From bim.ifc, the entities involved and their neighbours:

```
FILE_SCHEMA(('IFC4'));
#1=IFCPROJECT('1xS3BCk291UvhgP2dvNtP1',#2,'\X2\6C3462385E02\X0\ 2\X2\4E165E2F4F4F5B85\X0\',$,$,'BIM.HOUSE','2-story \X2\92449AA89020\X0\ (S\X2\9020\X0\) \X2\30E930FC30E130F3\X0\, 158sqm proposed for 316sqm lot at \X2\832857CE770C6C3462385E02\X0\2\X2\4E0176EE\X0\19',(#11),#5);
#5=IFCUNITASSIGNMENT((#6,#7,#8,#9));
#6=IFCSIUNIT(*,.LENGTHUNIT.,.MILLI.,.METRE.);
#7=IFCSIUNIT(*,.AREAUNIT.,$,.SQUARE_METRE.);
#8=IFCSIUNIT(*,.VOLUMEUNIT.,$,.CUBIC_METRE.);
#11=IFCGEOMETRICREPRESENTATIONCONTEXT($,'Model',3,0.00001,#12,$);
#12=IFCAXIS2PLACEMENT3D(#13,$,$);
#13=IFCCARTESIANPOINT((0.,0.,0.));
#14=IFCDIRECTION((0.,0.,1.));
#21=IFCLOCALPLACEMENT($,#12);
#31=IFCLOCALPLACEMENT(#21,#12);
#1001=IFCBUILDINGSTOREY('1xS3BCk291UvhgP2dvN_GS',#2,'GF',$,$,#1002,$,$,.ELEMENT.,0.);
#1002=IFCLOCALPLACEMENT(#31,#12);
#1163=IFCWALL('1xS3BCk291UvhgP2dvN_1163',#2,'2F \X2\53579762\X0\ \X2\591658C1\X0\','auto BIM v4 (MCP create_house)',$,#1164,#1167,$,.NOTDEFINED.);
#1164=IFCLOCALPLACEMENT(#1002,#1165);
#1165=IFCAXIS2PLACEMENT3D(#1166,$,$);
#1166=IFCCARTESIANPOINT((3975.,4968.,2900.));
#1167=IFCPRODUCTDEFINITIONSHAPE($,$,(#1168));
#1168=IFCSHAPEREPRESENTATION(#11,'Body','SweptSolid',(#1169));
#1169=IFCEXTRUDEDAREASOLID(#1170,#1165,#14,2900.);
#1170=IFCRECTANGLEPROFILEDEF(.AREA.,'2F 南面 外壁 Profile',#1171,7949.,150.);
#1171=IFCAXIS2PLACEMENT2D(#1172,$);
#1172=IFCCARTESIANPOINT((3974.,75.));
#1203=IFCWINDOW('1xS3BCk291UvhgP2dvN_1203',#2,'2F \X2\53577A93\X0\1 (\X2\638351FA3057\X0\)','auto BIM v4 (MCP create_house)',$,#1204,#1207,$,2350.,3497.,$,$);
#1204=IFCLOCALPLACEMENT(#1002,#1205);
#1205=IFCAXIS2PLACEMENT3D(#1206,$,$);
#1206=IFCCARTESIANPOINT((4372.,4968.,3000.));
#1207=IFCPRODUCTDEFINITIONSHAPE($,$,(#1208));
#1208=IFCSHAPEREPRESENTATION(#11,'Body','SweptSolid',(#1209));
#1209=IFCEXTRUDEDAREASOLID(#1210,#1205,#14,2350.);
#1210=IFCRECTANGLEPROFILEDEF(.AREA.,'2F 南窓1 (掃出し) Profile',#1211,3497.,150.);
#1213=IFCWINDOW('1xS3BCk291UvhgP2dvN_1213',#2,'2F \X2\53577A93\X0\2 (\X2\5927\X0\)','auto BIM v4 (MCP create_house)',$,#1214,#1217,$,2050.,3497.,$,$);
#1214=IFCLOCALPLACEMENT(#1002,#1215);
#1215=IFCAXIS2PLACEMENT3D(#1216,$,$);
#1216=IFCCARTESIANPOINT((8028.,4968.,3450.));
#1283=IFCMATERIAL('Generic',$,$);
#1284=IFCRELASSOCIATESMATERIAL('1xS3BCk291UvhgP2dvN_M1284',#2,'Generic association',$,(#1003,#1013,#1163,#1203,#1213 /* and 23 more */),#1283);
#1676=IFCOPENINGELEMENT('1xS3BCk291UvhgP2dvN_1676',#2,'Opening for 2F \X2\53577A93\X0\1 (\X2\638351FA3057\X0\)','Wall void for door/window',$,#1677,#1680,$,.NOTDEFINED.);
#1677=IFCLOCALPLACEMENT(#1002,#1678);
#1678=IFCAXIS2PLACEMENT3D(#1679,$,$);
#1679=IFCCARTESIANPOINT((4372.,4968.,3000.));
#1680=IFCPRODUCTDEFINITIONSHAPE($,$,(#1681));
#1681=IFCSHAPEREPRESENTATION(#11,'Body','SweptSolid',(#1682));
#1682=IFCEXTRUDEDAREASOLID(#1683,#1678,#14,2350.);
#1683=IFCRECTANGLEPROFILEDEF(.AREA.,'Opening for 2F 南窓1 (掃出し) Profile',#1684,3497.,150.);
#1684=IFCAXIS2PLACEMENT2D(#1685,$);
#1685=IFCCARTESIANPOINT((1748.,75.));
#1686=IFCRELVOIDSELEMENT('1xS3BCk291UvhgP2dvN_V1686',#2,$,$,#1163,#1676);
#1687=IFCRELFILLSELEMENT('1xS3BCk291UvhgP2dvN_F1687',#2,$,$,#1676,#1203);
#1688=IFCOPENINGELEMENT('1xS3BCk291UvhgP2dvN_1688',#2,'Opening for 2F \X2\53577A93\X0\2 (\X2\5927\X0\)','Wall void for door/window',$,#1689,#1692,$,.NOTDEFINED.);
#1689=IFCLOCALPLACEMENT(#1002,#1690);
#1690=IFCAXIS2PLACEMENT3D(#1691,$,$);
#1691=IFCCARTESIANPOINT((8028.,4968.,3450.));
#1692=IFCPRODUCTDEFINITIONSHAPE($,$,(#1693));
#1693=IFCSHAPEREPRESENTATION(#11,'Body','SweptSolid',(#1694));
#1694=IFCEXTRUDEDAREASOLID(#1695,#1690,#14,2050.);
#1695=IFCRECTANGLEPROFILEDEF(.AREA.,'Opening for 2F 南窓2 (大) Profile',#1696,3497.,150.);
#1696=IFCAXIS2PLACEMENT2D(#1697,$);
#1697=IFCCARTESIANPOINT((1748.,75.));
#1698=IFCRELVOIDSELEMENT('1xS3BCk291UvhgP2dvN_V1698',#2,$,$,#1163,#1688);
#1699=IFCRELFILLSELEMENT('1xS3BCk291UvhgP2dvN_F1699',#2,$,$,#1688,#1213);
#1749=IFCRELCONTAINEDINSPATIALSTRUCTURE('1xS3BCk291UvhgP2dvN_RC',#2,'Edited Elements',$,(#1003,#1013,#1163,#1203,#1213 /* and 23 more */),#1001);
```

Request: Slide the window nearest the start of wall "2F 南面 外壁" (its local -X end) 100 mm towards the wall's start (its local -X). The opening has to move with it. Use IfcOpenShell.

```python
import ifcopenshell
import ifcopenshell.api.geometry
import ifcopenshell.util.placement
import ifcopenshell.util.unit

model = ifcopenshell.open("bim.ifc")
unit_scale = ifcopenshell.util.unit.calculate_unit_scale(model)

window = model.by_guid("1xS3BCk291UvhgP2dvN_1203")
opening = window.FillsVoids[0].RelatingOpeningElement
wall = opening.VoidsElements[0].RelatingBuildingElement

wall_matrix = ifcopenshell.util.placement.get_local_placement(wall.ObjectPlacement)
shift = wall_matrix[:3, 0] * -0.1 / unit_scale
before = ifcopenshell.util.placement.get_local_placement(window.ObjectPlacement)[:3, 3].copy()

# The window is not placed relative to its opening, so move both.
for product in (opening, window):
    matrix = ifcopenshell.util.placement.get_local_placement(product.ObjectPlacement)
    matrix[:3, 3] += shift
    ifcopenshell.api.geometry.edit_object_placement(model, product=product, matrix=matrix, is_si=False)

after = ifcopenshell.util.placement.get_local_placement(window.ObjectPlacement)[:3, 3]
print("window moved by", (after - before).round(3) + 0.0)

model.write("bim_v2.ifc")
```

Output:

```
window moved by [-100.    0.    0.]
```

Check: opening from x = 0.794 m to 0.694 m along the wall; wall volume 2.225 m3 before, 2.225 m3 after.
